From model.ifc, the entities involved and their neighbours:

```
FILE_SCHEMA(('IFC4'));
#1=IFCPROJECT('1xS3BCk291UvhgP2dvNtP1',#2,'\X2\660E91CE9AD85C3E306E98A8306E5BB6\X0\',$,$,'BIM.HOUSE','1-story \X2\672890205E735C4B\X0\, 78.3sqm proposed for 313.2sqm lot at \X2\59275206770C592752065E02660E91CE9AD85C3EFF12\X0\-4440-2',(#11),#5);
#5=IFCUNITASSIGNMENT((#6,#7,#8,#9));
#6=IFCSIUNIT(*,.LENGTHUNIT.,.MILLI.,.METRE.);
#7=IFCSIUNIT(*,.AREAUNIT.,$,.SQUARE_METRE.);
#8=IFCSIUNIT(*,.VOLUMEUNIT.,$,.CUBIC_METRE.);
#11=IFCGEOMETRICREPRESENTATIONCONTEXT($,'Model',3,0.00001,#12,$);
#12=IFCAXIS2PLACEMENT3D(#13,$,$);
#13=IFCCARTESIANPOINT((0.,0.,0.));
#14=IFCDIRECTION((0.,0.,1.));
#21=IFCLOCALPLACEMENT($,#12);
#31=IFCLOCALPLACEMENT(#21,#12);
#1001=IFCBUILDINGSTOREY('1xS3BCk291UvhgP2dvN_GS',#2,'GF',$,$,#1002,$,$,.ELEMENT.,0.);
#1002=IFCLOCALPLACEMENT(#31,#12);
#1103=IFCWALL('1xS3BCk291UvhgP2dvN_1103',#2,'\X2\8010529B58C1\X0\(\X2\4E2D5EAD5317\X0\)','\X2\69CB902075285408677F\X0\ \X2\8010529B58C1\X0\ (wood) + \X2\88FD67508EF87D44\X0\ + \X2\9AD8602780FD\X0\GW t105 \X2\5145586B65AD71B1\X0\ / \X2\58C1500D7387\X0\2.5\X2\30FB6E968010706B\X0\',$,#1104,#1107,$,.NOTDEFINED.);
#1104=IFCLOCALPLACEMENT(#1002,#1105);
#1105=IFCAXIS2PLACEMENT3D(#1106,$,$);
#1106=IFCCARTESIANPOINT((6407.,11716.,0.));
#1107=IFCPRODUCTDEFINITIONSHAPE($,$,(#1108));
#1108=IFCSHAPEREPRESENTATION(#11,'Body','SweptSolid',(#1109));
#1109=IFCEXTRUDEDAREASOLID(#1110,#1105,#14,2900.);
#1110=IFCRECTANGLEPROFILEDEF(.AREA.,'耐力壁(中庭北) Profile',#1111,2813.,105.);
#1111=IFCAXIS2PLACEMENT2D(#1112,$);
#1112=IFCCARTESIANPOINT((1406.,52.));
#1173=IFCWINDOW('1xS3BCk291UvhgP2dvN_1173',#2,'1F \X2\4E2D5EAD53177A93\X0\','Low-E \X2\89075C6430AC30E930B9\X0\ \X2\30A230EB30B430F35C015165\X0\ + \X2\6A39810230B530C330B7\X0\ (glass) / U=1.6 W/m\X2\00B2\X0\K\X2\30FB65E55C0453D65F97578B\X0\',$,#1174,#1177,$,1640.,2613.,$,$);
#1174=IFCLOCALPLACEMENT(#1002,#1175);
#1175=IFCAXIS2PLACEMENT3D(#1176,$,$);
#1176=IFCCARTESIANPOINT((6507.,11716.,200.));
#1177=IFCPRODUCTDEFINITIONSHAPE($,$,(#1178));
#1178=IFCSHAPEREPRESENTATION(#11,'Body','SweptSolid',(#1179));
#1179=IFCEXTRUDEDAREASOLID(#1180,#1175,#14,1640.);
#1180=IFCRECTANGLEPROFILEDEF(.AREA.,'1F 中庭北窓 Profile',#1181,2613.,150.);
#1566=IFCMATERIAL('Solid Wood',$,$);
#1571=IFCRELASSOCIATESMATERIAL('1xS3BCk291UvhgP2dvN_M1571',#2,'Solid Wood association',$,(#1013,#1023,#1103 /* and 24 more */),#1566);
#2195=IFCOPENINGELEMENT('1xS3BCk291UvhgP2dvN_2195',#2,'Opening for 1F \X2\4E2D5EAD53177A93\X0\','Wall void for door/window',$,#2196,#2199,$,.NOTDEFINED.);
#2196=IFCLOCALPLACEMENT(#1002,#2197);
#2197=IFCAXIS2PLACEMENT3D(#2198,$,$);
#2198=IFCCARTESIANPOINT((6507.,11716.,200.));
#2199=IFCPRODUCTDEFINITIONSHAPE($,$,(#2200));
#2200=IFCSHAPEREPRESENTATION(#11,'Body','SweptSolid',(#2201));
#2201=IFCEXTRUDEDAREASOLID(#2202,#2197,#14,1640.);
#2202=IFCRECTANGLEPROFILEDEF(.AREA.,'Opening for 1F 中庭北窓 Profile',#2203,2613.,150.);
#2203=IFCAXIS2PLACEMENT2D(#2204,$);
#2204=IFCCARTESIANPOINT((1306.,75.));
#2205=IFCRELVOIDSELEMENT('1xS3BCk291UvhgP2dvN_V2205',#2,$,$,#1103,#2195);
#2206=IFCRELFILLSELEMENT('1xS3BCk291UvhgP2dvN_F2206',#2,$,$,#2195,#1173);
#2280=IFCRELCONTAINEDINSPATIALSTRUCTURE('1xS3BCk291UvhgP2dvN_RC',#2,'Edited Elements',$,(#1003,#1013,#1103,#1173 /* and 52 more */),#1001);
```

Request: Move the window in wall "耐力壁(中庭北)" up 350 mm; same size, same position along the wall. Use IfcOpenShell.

```python
import numpy as np
import ifcopenshell
import ifcopenshell.api.geometry
import ifcopenshell.util.placement
import ifcopenshell.util.unit

model = ifcopenshell.open("model.ifc")
unit_scale = ifcopenshell.util.unit.calculate_unit_scale(model)

window = model.by_guid("1xS3BCk291UvhgP2dvN_1173")
opening = window.FillsVoids[0].RelatingOpeningElement
dz = 0.35 / unit_scale

shift = np.array([0.0, 0.0, dz])
# The window is not placed relative to its opening, so move both.
for product in (opening, window):
    matrix = ifcopenshell.util.placement.get_local_placement(product.ObjectPlacement)
    matrix[:3, 3] += shift
    ifcopenshell.api.geometry.edit_object_placement(model, product=product, matrix=matrix, is_si=False)

print(f"moved by {dz * unit_scale:+.3f} m")

model.write("model_updated.ifc")
```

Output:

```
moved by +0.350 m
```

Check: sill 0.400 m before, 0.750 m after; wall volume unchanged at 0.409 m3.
